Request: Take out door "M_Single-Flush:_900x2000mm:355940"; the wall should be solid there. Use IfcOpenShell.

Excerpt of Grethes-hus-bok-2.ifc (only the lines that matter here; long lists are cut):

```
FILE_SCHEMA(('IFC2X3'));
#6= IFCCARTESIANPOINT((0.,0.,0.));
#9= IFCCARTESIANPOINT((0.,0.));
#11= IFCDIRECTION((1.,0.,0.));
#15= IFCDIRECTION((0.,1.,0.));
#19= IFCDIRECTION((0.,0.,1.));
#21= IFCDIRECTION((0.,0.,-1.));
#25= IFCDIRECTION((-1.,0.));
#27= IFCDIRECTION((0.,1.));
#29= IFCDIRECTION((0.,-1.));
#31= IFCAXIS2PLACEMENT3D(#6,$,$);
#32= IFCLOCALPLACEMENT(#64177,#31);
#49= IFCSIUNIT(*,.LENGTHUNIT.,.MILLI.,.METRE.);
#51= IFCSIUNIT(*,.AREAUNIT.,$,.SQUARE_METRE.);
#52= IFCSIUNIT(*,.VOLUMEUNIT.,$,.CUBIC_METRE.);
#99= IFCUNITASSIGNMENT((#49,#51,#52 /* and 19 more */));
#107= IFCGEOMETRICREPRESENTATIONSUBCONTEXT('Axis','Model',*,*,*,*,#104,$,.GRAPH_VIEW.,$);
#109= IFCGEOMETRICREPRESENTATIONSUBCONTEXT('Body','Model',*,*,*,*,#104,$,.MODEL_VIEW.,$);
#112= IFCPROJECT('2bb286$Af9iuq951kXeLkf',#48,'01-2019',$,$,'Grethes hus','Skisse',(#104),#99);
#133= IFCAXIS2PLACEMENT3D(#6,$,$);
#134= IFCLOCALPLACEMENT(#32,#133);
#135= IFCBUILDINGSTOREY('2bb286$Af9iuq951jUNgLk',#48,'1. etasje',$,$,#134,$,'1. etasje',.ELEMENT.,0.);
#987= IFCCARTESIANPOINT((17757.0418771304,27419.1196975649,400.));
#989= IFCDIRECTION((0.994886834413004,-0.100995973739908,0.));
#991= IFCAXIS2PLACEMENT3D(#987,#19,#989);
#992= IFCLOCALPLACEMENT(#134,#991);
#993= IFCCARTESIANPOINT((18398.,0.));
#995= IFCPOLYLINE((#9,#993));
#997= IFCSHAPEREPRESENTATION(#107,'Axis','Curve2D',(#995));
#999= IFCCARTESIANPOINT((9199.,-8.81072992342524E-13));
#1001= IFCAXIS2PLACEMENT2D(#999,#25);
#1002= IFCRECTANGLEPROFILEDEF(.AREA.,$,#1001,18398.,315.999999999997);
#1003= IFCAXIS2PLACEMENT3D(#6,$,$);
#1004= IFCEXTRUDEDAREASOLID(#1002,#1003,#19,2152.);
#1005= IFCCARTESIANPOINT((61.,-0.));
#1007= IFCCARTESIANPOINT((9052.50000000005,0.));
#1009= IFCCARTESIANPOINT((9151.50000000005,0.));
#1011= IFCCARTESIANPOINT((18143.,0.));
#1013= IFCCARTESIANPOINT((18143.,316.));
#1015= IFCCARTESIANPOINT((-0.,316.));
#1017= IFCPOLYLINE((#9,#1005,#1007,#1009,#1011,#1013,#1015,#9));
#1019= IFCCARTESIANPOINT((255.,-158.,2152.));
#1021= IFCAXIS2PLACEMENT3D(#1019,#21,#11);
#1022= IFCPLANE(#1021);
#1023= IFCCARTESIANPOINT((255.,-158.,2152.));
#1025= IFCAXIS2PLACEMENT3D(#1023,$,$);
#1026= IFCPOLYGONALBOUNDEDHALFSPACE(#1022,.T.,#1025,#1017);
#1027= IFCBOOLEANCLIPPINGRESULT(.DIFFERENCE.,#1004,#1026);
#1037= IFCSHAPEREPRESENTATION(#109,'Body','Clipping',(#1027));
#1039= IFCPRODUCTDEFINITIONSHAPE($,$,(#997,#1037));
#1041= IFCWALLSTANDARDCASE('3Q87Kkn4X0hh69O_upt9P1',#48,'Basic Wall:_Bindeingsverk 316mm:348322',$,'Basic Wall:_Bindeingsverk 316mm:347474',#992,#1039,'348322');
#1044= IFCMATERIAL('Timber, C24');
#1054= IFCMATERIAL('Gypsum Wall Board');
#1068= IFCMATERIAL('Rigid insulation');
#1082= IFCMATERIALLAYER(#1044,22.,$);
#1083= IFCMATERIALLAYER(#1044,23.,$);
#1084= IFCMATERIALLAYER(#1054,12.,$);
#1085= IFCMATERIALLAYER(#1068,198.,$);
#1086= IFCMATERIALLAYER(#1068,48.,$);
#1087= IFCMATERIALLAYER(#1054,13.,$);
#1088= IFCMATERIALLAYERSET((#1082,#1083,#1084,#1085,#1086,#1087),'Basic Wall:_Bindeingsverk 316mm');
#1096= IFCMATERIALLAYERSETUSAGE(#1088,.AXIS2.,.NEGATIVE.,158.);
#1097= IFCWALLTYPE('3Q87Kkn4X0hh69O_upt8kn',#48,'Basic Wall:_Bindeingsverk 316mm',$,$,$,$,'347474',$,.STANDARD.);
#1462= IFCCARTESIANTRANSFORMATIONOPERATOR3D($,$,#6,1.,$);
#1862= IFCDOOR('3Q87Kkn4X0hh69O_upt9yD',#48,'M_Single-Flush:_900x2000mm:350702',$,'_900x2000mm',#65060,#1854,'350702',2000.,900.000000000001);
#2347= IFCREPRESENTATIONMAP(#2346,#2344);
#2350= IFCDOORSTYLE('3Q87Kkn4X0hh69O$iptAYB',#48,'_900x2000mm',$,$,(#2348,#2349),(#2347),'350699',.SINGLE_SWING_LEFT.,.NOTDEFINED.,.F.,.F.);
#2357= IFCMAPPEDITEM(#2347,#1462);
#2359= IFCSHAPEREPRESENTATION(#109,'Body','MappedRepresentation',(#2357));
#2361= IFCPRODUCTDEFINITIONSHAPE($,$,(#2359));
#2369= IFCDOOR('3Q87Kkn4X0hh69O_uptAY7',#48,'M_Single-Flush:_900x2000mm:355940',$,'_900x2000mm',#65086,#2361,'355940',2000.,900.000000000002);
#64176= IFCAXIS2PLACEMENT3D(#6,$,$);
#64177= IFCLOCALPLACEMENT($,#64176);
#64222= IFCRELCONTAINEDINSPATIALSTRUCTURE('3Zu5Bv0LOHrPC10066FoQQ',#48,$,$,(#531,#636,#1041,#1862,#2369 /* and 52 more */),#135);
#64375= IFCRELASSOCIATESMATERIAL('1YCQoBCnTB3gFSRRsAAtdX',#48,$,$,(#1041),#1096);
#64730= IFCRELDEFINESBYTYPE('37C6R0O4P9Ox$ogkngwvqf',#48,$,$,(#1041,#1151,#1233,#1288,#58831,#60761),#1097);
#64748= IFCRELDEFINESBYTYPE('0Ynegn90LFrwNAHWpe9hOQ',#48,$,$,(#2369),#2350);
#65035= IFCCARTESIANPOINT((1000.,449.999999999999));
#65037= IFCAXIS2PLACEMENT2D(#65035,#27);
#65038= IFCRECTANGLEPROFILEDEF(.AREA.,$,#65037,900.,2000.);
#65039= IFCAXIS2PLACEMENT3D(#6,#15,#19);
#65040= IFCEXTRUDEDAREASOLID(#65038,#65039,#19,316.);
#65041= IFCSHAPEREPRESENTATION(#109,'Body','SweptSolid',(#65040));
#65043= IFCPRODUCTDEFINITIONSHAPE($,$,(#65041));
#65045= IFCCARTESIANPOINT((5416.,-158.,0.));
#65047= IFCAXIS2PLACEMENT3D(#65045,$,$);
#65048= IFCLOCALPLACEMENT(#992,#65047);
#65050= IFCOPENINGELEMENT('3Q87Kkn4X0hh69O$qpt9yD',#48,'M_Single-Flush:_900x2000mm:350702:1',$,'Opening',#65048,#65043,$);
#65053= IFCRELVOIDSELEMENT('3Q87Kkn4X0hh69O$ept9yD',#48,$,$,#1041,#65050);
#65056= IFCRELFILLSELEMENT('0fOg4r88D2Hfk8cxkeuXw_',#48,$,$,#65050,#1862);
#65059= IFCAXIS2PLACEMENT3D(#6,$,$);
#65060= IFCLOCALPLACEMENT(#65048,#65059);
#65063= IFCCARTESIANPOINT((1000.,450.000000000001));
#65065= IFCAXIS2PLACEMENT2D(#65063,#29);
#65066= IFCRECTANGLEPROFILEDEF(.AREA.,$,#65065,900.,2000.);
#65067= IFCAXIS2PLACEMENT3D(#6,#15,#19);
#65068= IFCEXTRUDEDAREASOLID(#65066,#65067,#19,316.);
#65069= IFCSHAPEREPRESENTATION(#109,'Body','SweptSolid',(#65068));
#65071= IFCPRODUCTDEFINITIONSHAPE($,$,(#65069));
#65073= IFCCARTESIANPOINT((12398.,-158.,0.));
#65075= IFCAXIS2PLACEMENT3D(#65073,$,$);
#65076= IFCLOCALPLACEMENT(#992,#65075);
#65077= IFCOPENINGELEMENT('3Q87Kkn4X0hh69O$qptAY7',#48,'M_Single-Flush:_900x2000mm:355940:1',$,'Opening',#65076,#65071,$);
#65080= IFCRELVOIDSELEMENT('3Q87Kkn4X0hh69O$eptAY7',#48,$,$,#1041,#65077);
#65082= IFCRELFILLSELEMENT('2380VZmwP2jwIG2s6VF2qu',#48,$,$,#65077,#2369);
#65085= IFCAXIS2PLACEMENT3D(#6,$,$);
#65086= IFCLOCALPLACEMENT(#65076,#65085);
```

```python
import ifcopenshell
import ifcopenshell.api.feature
import ifcopenshell.api.root
import ifcopenshell.geom
import ifcopenshell.util.shape

model = ifcopenshell.open("Grethes-hus-bok-2.ifc")
settings = ifcopenshell.geom.settings()


def volume(element):
    """Net volume in cubic metres, openings subtracted."""
    shape = ifcopenshell.geom.create_shape(settings, element)
    return ifcopenshell.util.shape.get_volume(shape.geometry)


door = model.by_guid("3Q87Kkn4X0hh69O_uptAY7")
opening = door.FillsVoids[0].RelatingOpeningElement
wall = opening.VoidsElements[0].RelatingBuildingElement
before = volume(wall)

ifcopenshell.api.root.remove_product(model, product=door)
ifcopenshell.api.feature.remove_feature(model, feature=opening)

after = volume(wall)

print(f"wall volume {before:.3f} -> {after:.3f} m3")

model.write("Grethes-hus-bok-2_updated.ifc")
```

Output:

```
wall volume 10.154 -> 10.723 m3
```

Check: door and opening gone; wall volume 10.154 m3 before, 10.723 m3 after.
